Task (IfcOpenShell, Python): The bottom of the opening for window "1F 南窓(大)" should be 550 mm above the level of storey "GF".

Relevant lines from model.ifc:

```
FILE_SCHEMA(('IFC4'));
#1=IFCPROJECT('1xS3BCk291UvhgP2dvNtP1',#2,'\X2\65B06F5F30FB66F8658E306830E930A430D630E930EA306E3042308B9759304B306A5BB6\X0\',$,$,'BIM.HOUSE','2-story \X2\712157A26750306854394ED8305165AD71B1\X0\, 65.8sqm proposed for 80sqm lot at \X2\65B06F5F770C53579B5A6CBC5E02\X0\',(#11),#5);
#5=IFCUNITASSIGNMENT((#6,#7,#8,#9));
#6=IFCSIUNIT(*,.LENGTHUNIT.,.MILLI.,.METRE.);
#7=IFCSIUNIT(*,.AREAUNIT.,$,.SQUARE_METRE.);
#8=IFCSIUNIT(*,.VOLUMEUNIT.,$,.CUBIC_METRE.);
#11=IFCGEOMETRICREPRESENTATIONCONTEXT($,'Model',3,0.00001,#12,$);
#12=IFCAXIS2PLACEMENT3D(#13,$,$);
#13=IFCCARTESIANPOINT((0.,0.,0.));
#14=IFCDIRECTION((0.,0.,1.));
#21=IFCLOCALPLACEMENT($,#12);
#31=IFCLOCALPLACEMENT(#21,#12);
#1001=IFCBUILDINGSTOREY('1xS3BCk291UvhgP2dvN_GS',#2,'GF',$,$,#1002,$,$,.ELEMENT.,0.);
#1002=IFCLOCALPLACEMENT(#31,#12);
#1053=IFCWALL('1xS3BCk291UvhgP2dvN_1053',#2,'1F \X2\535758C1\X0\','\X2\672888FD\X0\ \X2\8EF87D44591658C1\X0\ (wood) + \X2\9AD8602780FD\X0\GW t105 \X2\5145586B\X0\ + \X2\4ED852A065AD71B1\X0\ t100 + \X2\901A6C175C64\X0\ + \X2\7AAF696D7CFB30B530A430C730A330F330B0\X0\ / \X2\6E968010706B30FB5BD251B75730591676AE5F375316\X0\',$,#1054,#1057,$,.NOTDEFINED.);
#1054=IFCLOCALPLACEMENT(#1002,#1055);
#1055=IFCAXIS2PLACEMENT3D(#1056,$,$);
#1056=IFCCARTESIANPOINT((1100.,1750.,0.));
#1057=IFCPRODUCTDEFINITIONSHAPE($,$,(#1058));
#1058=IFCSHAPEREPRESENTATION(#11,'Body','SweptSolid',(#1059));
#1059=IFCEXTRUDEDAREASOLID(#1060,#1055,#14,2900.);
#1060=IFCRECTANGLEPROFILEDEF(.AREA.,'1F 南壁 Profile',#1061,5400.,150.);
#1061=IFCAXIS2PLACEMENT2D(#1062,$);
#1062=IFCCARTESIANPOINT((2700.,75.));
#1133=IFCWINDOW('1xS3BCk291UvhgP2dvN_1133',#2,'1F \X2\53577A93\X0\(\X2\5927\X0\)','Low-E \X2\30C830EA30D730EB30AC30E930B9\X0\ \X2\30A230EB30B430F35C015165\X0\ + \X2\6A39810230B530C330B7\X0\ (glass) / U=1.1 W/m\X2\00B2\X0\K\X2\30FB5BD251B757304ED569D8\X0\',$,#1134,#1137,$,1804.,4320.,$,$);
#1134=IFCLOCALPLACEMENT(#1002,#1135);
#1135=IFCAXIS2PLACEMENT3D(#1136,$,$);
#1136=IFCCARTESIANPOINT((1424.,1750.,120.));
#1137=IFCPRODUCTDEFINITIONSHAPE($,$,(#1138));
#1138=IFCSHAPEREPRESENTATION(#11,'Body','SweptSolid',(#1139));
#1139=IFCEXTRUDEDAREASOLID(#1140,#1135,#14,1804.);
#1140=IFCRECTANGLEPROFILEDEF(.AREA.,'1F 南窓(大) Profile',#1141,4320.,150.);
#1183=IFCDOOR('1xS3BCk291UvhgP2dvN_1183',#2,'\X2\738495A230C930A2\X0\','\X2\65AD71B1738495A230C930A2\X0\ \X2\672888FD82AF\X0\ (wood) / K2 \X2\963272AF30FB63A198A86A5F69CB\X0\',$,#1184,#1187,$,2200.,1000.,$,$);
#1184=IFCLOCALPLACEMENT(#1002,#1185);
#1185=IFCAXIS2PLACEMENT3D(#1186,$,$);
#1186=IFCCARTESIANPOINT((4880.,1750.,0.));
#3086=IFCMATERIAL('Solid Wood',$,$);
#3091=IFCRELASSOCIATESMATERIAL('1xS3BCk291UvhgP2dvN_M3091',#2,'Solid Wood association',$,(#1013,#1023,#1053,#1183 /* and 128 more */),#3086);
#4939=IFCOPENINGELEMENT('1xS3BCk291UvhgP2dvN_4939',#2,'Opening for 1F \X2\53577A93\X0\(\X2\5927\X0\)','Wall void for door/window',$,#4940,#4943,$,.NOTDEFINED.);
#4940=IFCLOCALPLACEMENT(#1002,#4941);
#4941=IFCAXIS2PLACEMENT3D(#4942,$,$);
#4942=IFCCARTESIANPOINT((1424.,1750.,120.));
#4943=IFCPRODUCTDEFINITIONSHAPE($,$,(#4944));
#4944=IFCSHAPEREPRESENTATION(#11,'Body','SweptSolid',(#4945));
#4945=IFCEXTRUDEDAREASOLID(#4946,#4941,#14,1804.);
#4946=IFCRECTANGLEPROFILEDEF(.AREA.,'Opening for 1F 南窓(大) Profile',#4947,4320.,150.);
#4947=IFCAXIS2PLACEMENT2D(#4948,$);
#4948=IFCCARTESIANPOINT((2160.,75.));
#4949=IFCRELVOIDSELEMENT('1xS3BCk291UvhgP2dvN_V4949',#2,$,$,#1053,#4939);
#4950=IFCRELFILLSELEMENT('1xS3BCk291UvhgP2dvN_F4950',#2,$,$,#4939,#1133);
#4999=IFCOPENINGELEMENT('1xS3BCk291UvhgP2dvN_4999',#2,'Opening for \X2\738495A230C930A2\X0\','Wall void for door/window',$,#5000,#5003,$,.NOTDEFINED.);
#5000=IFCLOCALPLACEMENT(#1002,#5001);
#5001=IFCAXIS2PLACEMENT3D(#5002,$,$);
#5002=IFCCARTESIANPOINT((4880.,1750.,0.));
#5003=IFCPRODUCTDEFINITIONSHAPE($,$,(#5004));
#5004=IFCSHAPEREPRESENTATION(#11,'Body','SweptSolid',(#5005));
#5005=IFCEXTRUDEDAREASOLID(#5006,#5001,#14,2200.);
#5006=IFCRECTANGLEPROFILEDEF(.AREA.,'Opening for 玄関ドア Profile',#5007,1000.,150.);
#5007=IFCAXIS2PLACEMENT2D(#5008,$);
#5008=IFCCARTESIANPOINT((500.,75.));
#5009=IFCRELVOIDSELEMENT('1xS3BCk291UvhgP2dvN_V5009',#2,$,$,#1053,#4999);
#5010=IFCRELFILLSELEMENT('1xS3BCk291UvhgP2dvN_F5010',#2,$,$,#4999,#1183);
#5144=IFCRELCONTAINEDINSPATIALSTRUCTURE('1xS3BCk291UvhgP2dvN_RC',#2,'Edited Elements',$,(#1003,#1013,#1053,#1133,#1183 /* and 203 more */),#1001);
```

```python
import numpy as np
import ifcopenshell
import ifcopenshell.api.geometry
import ifcopenshell.geom
import ifcopenshell.util.element
import ifcopenshell.util.placement
import ifcopenshell.util.shape
import ifcopenshell.util.unit

model = ifcopenshell.open("model.ifc")
unit_scale = ifcopenshell.util.unit.calculate_unit_scale(model)

window = model.by_id(1133)
opening = window.FillsVoids[0].RelatingOpeningElement
storey = ifcopenshell.util.element.get_container(window, ifc_class="IfcBuildingStorey")
level = ifcopenshell.util.placement.get_local_placement(storey.ObjectPlacement)[2, 3]

# The opening's origin need not be at the sill, so measure its lowest point.
shape = ifcopenshell.geom.create_shape(ifcopenshell.geom.settings(), opening)
bottom = ifcopenshell.util.shape.get_shape_bottom_elevation(shape, shape.geometry) / unit_scale
dz = level + 550.0 - bottom

shift = np.array([0.0, 0.0, dz])
# The window is not placed relative to its opening, so move both.
for product in (opening, window):
    matrix = ifcopenshell.util.placement.get_local_placement(product.ObjectPlacement)
    matrix[:3, 3] += shift
    ifcopenshell.api.geometry.edit_object_placement(model, product=product, matrix=matrix, is_si=False)

print(f"moved by {dz * unit_scale:+.3f} m")

model.write("model_edited.ifc")
```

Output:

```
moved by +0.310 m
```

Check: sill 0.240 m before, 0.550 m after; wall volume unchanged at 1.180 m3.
